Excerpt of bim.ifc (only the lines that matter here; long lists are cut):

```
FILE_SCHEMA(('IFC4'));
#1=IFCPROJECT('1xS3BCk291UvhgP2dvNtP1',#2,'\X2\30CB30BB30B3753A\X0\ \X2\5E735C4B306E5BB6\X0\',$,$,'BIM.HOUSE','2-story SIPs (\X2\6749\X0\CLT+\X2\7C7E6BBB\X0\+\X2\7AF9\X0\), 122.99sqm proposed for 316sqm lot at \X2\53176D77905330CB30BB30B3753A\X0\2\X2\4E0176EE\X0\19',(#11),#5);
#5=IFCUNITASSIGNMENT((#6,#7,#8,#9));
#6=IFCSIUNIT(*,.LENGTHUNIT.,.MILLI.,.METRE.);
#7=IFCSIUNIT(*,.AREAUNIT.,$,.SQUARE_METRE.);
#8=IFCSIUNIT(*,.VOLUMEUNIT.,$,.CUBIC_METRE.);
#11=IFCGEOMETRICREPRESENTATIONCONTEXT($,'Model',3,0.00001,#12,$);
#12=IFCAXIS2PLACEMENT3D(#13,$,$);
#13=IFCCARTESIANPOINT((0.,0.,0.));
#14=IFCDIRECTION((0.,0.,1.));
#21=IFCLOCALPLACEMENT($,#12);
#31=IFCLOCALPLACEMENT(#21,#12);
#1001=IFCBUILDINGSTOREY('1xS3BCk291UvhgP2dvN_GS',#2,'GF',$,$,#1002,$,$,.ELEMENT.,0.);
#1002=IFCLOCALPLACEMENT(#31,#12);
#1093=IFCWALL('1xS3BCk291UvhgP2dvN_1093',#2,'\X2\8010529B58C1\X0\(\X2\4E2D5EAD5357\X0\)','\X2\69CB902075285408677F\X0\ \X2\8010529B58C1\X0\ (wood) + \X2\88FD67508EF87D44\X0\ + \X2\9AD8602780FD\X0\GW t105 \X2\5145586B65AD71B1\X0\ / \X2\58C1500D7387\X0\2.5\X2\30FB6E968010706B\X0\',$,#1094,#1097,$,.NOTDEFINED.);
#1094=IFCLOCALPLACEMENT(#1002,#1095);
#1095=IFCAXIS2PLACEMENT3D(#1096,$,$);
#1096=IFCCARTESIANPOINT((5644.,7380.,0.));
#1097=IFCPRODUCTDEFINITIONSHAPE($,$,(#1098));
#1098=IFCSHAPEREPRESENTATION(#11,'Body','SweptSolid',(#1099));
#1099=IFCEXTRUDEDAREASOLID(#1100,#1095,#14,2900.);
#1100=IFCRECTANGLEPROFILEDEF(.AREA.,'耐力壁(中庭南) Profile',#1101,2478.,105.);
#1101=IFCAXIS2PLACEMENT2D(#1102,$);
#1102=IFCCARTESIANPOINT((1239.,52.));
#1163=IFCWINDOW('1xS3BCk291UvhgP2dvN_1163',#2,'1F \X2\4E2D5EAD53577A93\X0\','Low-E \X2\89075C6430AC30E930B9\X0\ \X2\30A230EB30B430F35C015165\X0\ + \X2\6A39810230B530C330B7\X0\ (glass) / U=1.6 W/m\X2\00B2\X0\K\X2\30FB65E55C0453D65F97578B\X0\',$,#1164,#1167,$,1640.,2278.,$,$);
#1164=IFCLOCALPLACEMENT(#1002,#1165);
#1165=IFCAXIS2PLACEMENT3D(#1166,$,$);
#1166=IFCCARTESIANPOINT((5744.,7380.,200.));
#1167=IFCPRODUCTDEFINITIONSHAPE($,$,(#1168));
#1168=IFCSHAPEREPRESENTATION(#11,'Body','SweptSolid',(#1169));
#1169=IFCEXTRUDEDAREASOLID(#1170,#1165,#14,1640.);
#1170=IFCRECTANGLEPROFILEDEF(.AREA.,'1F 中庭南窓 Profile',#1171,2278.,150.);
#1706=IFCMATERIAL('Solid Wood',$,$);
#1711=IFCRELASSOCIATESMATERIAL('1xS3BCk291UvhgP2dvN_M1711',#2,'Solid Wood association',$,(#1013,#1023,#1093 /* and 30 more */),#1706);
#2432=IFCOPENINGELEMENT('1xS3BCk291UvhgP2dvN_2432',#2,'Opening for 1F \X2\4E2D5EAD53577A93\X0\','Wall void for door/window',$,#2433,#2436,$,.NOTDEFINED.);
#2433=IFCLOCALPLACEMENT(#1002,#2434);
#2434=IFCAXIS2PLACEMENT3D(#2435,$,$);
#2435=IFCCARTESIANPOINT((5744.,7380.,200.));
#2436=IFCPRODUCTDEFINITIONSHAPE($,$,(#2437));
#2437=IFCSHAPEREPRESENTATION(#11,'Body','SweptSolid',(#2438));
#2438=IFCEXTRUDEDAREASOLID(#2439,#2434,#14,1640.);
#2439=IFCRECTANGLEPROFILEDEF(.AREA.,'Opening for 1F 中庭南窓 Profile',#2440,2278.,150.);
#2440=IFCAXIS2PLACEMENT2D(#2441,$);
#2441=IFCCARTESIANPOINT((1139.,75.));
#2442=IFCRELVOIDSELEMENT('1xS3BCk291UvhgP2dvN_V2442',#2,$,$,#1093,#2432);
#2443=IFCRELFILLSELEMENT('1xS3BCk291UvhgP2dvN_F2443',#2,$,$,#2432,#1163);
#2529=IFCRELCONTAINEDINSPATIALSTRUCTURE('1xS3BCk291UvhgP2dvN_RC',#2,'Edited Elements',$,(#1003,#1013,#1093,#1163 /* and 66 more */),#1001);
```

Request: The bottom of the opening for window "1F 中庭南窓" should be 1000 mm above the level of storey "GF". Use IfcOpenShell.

```python
import numpy as np
import ifcopenshell
import ifcopenshell.api.geometry
import ifcopenshell.geom
import ifcopenshell.util.element
import ifcopenshell.util.placement
import ifcopenshell.util.shape
import ifcopenshell.util.unit

model = ifcopenshell.open("bim.ifc")
unit_scale = ifcopenshell.util.unit.calculate_unit_scale(model)

window = model.by_guid("1xS3BCk291UvhgP2dvN_1163")
opening = window.FillsVoids[0].RelatingOpeningElement
storey = ifcopenshell.util.element.get_container(window, ifc_class="IfcBuildingStorey")
level = ifcopenshell.util.placement.get_local_placement(storey.ObjectPlacement)[2, 3]

# The opening's origin need not be at the sill, so measure its lowest point.
shape = ifcopenshell.geom.create_shape(ifcopenshell.geom.settings(), opening)
bottom = ifcopenshell.util.shape.get_shape_bottom_elevation(shape, shape.geometry) / unit_scale
dz = level + 1 / unit_scale - bottom

shift = np.array([0.0, 0.0, dz])
# The window is not placed relative to its opening, so move both.
for product in (opening, window):
    matrix = ifcopenshell.util.placement.get_local_placement(product.ObjectPlacement)
    matrix[:3, 3] += shift
    ifcopenshell.api.geometry.edit_object_placement(model, product=product, matrix=matrix, is_si=False)

print(f"moved by {dz * unit_scale:+.3f} m")

model.write("bim_rev.ifc")
```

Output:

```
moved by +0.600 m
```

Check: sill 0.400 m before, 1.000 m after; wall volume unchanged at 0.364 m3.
